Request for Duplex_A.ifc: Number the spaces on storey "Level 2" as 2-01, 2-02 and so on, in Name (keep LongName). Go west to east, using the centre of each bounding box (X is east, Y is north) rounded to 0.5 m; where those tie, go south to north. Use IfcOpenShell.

First a look at what the model holds.

```python
import ifcopenshell
import ifcopenshell.util.element
import ifcopenshell.util.placement

model = ifcopenshell.open("Duplex_A.ifc")
print(model.schema)
storey = next(s for s in model.by_type("IfcBuildingStorey") if s.Name == "Level 2")
spaces = [e for e in ifcopenshell.util.element.get_decomposition(storey) if e.is_a("IfcSpace")]
for e in sorted(spaces, key=lambda e: e.id()):
    origin = ifcopenshell.util.placement.get_local_placement(e.ObjectPlacement)[:3, 3]
    print(e.id(), e.Name, e.LongName, origin.round(2) + 0.0, sep=" | ")
```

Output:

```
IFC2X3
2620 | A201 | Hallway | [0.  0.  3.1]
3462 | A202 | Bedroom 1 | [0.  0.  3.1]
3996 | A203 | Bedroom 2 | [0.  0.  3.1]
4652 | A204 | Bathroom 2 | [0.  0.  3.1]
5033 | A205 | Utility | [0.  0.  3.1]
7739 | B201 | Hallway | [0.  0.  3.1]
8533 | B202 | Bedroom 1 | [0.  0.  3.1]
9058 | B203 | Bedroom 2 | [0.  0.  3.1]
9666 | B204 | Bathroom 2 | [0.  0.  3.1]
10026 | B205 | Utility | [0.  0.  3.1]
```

```python
import ifcopenshell
import ifcopenshell.geom
import ifcopenshell.util.element
import ifcopenshell.util.shape

model = ifcopenshell.open("Duplex_A.ifc")
settings = ifcopenshell.geom.settings()
settings.set("use-world-coords", True)


def centre(element):
    shape = ifcopenshell.geom.create_shape(settings, element)
    return ifcopenshell.util.shape.get_bbox_centroid(shape.geometry)


storey = next(s for s in model.by_type("IfcBuildingStorey") if s.Name == "Level 2")
spaces = [e for e in ifcopenshell.util.element.get_decomposition(storey) if e.is_a("IfcSpace")]

# Insertion points can sit at a corner or the storey origin, so sort by the geometry (in metres).
centres = {e: centre(e) for e in spaces}
spaces.sort(key=lambda e: (round(centres[e][0] / 0.5), centres[e][1]))

for i, e in enumerate(spaces, start=1):
    number = f"2-{i:02d}"
    e.Name = number
    print(e.id(), number)

model.write("Duplex_A_edited.ifc")
```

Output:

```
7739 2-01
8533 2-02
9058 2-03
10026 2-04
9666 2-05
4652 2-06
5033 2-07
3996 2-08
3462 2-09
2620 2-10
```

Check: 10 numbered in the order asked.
